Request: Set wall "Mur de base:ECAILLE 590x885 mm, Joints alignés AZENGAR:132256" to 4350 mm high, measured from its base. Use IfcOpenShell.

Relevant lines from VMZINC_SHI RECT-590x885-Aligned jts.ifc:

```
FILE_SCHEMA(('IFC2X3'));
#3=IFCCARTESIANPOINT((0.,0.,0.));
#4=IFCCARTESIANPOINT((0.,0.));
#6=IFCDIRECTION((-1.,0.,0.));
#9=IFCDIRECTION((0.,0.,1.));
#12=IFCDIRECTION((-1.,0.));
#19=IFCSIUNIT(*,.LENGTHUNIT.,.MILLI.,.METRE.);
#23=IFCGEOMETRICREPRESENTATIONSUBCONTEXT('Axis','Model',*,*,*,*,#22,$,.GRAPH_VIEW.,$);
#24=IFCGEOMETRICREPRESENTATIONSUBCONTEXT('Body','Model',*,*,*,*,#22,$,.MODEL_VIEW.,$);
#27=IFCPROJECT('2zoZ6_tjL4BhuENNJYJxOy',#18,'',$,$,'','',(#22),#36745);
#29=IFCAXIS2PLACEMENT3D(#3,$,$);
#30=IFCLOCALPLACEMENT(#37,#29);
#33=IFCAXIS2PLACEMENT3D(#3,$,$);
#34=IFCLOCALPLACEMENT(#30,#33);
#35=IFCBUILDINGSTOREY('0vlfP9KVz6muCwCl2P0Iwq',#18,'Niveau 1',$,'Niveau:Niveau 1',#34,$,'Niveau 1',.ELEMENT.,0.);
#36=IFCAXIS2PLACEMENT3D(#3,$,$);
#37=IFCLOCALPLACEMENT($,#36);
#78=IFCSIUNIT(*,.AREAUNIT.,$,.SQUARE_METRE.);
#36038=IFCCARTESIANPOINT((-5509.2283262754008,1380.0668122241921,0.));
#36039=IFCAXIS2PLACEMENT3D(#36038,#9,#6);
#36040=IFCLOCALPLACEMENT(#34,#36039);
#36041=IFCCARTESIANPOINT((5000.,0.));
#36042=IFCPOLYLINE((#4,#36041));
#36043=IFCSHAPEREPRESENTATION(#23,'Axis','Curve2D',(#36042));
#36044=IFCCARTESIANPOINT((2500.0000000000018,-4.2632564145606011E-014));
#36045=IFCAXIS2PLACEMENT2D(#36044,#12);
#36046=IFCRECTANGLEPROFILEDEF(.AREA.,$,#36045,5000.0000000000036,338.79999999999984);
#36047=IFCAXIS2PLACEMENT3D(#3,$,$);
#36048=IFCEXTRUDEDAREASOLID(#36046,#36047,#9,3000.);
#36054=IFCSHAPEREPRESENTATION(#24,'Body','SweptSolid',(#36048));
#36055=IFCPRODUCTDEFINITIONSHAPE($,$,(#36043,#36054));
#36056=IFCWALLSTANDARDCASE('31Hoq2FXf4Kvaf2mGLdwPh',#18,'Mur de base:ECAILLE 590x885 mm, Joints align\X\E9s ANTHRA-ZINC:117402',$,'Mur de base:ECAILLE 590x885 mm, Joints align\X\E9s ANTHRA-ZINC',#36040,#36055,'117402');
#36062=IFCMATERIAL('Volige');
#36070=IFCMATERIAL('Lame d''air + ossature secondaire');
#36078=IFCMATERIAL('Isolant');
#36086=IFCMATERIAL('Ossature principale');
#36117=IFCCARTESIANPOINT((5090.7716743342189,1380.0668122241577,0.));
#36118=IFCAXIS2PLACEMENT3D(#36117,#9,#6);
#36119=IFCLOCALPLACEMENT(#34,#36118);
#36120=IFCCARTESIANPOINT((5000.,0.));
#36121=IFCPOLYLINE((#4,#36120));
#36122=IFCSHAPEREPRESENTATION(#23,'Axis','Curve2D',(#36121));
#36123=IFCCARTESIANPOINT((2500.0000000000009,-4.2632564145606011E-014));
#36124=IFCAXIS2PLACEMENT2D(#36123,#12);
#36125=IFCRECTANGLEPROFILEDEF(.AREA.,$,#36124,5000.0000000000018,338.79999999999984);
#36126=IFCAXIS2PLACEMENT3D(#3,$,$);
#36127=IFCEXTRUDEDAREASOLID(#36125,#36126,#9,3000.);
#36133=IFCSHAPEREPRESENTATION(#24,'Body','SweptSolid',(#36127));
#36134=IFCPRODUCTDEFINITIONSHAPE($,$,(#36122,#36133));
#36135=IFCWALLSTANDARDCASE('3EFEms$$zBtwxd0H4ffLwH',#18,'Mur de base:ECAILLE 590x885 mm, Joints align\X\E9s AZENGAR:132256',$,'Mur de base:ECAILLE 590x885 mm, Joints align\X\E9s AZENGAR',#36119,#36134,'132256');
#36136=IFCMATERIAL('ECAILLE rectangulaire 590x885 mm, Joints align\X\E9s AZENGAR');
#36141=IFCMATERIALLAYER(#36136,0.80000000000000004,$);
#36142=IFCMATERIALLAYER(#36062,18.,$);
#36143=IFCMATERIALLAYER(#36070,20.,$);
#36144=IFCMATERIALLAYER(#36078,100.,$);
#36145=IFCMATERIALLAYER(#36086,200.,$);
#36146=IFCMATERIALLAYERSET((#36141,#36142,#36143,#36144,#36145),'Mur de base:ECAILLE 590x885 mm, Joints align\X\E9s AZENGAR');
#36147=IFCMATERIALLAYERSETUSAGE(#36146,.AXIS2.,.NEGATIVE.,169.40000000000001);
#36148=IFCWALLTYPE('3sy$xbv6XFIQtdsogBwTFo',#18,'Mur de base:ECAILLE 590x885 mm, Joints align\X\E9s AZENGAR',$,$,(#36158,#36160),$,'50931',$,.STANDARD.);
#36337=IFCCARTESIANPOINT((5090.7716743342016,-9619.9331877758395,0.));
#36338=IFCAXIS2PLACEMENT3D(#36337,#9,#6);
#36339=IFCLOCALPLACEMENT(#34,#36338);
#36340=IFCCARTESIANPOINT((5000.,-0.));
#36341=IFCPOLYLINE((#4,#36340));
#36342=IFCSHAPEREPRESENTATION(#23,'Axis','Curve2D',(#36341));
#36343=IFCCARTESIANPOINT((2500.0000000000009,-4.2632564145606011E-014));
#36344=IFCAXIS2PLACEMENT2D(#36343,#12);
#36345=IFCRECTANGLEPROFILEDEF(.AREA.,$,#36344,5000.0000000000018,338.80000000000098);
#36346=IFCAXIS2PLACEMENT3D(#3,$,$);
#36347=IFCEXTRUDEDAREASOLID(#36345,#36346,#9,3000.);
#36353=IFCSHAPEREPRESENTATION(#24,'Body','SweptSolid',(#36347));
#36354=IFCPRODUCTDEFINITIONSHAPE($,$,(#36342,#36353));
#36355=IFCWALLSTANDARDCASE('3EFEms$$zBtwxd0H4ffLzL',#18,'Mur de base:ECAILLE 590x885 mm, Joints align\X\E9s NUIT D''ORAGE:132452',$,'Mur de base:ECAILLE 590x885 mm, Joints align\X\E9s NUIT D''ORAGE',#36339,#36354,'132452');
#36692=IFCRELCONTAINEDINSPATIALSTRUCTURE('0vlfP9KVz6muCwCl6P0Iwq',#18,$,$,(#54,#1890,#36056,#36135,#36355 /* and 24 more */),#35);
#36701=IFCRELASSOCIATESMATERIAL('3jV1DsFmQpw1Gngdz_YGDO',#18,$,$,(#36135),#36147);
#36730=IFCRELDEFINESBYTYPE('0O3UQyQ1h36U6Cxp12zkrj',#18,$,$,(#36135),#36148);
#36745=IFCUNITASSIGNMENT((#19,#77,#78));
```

```python
import ifcopenshell
import ifcopenshell.geom
import ifcopenshell.util.representation
import ifcopenshell.util.shape
import ifcopenshell.util.unit

model = ifcopenshell.open("VMZINC_SHI RECT-590x885-Aligned jts.ifc")
unit_scale = ifcopenshell.util.unit.calculate_unit_scale(model)
settings = ifcopenshell.geom.settings()


def volume(element):
    """Net volume in cubic metres, openings subtracted."""
    shape = ifcopenshell.geom.create_shape(settings, element)
    return ifcopenshell.util.shape.get_volume(shape.geometry)


wall = model.by_guid("3EFEms$$zBtwxd0H4ffLwH")
before = volume(wall)

body = ifcopenshell.util.representation.get_representation(wall, "Model", "Body")
solid = body.Items[0]
old_height = solid.Depth
solid.Depth = 4.35 / unit_scale
after = volume(wall)

print(f"height {old_height:g} -> {solid.Depth:g}, volume {before:.3f} -> {after:.3f} m3")

model.write("VMZINC_SHI RECT-590x885-Aligned jts_rev.ifc")
```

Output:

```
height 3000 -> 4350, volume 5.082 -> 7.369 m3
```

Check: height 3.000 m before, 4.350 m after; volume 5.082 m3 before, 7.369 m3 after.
